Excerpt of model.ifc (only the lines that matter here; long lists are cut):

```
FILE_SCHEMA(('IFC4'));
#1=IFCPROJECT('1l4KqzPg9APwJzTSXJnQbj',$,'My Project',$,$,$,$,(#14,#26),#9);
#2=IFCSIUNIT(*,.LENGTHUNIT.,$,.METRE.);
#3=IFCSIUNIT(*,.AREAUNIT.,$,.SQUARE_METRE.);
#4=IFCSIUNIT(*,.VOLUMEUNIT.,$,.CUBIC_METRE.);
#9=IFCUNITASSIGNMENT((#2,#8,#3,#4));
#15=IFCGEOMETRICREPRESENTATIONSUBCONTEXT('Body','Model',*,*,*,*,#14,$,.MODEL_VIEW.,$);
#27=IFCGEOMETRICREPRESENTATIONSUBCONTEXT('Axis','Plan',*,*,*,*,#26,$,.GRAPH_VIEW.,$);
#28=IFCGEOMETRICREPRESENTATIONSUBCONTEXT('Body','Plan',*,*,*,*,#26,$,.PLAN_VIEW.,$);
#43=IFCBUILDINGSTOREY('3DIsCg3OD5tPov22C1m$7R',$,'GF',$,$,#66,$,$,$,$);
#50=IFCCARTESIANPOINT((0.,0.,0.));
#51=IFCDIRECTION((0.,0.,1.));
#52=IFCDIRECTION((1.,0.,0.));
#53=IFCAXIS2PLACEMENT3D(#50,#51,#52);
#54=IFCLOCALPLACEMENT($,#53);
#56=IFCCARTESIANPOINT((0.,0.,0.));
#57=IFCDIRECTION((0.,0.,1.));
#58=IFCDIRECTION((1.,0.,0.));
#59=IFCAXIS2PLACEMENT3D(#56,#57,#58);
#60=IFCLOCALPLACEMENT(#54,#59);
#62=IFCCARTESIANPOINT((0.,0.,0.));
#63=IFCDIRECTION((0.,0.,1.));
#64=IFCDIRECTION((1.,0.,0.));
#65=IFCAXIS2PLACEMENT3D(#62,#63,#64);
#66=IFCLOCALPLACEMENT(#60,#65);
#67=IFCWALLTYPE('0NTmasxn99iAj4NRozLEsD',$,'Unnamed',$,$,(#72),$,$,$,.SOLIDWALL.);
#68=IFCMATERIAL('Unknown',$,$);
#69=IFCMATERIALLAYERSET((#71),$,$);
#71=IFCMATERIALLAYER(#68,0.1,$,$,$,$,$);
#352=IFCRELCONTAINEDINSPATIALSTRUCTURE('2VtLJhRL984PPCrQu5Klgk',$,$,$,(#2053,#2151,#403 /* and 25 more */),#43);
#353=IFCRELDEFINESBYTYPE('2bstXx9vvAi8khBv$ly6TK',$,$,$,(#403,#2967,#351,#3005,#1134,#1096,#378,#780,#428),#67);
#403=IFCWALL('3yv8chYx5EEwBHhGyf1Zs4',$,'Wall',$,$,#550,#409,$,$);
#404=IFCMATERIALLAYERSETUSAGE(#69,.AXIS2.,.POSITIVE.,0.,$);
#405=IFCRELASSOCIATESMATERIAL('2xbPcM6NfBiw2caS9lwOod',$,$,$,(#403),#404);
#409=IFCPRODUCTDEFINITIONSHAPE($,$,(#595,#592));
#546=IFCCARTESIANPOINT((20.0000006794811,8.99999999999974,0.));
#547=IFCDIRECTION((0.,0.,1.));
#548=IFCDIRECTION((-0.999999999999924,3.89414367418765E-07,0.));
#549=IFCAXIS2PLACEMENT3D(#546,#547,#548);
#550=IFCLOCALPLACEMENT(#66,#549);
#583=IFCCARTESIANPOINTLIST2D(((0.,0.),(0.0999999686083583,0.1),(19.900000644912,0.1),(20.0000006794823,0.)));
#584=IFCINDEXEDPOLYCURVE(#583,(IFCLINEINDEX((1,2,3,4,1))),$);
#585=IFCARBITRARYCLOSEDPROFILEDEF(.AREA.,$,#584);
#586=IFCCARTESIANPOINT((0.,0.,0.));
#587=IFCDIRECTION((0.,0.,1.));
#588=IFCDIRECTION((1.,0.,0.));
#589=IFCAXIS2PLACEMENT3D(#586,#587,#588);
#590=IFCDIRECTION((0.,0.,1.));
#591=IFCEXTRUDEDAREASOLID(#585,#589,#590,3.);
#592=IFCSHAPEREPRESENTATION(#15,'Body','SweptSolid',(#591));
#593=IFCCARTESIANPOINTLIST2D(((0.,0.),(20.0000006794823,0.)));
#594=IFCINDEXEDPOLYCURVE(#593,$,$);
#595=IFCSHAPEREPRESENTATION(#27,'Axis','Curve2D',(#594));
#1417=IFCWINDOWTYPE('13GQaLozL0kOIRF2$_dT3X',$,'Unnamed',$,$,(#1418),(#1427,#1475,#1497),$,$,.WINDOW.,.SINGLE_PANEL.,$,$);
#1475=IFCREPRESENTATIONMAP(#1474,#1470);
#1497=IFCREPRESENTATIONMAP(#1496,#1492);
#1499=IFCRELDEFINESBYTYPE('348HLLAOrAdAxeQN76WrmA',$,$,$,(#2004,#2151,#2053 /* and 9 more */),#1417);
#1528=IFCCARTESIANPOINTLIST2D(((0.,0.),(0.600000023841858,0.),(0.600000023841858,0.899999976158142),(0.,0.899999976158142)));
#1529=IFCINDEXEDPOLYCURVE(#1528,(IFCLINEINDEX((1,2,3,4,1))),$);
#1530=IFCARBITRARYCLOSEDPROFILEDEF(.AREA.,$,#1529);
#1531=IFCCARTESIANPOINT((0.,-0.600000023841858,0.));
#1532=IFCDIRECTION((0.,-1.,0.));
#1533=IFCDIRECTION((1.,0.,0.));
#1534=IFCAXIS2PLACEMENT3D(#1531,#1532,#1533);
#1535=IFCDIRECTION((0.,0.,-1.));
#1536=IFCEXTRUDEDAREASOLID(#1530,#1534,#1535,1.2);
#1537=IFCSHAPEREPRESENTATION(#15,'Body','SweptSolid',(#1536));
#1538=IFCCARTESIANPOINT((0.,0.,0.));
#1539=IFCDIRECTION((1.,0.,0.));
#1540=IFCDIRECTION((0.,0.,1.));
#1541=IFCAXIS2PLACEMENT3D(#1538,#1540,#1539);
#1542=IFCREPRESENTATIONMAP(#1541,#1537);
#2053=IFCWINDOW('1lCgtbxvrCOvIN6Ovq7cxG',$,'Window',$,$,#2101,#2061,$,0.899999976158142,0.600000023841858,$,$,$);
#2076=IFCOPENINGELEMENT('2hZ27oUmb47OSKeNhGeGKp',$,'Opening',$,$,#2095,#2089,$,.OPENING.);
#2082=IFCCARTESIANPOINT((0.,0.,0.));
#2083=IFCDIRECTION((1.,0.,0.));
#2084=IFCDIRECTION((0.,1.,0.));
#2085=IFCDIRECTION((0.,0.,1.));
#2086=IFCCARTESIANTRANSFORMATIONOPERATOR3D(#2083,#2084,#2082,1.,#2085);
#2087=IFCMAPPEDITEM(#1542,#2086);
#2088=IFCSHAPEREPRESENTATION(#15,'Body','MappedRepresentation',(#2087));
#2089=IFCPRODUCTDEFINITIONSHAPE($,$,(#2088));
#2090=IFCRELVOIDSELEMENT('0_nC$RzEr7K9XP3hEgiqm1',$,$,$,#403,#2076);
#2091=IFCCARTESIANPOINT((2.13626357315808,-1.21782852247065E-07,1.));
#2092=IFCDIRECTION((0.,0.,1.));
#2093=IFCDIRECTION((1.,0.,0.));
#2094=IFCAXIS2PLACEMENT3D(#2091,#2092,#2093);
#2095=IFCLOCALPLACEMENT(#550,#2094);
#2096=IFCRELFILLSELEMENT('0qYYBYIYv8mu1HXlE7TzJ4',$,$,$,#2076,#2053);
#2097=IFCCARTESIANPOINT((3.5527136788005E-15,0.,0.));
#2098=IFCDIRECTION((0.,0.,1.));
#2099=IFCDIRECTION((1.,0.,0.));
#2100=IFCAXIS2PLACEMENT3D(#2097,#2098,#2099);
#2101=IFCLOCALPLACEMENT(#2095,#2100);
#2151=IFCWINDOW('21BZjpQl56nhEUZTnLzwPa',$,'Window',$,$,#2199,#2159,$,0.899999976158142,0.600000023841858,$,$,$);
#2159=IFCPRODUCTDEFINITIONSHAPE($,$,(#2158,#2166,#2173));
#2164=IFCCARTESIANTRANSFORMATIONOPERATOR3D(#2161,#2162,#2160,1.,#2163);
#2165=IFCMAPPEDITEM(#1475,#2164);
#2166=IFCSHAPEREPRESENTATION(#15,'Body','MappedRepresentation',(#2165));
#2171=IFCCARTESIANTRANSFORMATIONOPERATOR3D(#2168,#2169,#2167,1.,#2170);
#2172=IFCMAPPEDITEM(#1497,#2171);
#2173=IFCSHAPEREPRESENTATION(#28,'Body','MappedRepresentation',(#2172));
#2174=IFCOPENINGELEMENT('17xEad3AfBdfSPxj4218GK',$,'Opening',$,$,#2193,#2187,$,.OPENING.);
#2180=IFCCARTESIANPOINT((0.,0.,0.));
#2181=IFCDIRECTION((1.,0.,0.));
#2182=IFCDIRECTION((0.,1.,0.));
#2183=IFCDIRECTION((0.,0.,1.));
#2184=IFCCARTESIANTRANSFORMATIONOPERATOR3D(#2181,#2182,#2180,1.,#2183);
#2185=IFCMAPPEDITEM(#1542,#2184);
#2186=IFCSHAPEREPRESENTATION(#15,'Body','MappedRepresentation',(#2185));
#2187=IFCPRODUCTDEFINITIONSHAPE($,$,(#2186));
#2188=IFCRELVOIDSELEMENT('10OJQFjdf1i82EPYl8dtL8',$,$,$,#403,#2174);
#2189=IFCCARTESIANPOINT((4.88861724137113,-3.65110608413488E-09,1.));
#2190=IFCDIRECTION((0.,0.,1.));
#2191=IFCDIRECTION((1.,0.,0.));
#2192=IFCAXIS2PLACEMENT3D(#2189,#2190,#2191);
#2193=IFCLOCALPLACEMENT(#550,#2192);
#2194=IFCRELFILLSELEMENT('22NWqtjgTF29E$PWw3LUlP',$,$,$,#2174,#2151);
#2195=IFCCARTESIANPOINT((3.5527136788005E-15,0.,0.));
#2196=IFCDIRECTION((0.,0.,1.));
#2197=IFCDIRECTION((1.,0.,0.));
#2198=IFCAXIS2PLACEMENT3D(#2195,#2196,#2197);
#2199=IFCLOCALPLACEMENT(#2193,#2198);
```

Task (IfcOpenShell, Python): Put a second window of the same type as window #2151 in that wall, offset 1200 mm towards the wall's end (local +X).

```python
import ifcopenshell
import ifcopenshell.api.feature
import ifcopenshell.api.geometry
import ifcopenshell.api.root
import ifcopenshell.geom
import ifcopenshell.util.element
import ifcopenshell.util.placement
import ifcopenshell.util.shape

model = ifcopenshell.open("model.ifc")
settings = ifcopenshell.geom.settings()


def volume(element):
    """Net volume in cubic metres, openings subtracted."""
    shape = ifcopenshell.geom.create_shape(settings, element)
    return ifcopenshell.util.shape.get_volume(shape.geometry)


window = model.by_id(2151)
opening = window.FillsVoids[0].RelatingOpeningElement
wall = opening.VoidsElements[0].RelatingBuildingElement
before = volume(wall)
shift = ifcopenshell.util.placement.get_local_placement(wall.ObjectPlacement)[:3, 0] * 1.2

# copy_class copies the void relationship, type, container and properties, but no geometry.
new_opening = ifcopenshell.api.root.copy_class(model, product=opening)
new_opening.Representation = ifcopenshell.util.element.copy_deep(
    model, opening.Representation, exclude=["IfcGeometricRepresentationContext", "IfcRepresentationMap"]
)
new_window = ifcopenshell.api.root.copy_class(model, product=window)
new_window.Representation = ifcopenshell.util.element.copy_deep(
    model, window.Representation, exclude=["IfcGeometricRepresentationContext", "IfcRepresentationMap"]
)
ifcopenshell.api.feature.add_filling(model, opening=new_opening, element=new_window)

for old, new in ((opening, new_opening), (window, new_window)):
    matrix = ifcopenshell.util.placement.get_local_placement(old.ObjectPlacement)
    matrix[:3, 3] += shift
    ifcopenshell.api.geometry.edit_object_placement(model, product=new, matrix=matrix, is_si=False)

after = volume(wall)

print(f"wall volume {before:.3f} -> {after:.3f} m3")

model.write("model_rev.ifc")
```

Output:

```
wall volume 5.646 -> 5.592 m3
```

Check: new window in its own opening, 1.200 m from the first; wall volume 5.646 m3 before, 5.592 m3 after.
